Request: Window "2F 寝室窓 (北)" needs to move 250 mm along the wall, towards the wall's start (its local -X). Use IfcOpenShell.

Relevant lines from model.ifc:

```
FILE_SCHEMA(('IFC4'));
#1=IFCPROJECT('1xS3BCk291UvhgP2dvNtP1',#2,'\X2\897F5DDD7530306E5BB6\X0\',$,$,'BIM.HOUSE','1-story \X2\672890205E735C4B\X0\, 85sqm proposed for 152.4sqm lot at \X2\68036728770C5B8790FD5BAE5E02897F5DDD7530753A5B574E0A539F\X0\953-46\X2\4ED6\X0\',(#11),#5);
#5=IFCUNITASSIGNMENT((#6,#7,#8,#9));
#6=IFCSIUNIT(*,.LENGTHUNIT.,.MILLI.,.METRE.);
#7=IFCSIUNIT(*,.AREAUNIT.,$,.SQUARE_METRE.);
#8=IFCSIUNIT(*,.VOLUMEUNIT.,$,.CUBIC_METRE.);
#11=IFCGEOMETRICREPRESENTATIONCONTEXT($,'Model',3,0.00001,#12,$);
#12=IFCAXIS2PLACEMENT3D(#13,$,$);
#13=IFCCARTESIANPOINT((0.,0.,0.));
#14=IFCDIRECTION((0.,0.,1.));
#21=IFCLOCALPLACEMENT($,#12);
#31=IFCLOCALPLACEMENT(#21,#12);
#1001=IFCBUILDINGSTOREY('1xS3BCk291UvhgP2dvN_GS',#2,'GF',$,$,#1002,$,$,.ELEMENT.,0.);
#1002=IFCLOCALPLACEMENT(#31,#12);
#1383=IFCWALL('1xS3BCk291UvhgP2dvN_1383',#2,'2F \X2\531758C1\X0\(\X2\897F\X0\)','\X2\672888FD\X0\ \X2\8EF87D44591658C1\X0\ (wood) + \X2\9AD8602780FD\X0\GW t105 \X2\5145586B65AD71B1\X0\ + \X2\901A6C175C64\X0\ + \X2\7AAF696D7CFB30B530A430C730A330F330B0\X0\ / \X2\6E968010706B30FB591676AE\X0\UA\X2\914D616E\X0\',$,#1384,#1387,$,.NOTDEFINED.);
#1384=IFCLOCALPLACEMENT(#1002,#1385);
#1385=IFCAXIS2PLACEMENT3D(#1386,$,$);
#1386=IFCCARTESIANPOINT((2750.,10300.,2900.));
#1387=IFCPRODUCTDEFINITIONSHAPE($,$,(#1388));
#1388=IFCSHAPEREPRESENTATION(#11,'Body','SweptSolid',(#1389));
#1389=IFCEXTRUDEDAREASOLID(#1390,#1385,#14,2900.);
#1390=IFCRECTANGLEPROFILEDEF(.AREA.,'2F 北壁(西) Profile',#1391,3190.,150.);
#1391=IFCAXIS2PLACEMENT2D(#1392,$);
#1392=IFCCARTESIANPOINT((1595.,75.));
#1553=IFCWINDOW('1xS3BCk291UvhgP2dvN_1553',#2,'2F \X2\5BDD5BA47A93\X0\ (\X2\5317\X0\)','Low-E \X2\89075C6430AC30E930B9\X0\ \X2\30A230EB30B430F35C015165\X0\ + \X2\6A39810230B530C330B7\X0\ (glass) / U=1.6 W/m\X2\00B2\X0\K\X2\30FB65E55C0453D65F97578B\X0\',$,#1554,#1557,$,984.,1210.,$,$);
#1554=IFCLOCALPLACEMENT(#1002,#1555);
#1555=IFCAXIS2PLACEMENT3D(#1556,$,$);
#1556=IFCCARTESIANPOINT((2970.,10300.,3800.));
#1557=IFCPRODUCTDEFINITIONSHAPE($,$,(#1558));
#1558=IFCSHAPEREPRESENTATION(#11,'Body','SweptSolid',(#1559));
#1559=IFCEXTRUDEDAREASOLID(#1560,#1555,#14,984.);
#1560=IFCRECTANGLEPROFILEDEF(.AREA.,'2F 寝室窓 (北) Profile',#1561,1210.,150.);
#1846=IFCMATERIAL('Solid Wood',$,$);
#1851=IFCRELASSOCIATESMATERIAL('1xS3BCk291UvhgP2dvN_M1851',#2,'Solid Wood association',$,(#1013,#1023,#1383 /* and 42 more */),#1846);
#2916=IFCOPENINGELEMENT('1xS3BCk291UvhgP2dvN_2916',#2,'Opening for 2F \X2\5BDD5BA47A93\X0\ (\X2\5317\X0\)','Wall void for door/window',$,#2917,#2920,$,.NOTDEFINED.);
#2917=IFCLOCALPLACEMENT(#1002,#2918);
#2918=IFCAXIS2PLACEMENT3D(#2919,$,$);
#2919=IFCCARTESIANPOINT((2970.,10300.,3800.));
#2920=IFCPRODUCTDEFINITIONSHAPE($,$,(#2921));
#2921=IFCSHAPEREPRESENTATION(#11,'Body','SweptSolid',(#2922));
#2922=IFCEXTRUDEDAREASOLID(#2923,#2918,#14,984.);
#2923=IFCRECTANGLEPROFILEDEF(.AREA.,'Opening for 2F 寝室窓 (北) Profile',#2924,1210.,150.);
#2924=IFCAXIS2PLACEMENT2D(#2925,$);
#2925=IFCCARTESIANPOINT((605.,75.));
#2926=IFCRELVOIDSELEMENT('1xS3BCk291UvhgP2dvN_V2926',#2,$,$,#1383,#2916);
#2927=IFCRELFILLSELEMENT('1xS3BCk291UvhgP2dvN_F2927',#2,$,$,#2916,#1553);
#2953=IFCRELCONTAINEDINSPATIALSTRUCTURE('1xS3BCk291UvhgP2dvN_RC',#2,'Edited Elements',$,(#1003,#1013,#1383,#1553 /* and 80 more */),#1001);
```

```python
import ifcopenshell
import ifcopenshell.api.geometry
import ifcopenshell.util.placement
import ifcopenshell.util.unit

model = ifcopenshell.open("model.ifc")
unit_scale = ifcopenshell.util.unit.calculate_unit_scale(model)

window = model.by_id(1553)
opening = window.FillsVoids[0].RelatingOpeningElement
wall = opening.VoidsElements[0].RelatingBuildingElement

wall_matrix = ifcopenshell.util.placement.get_local_placement(wall.ObjectPlacement)
shift = wall_matrix[:3, 0] * -0.25 / unit_scale
before = ifcopenshell.util.placement.get_local_placement(window.ObjectPlacement)[:3, 3].copy()

# The window is not placed relative to its opening, so move both.
for product in (opening, window):
    matrix = ifcopenshell.util.placement.get_local_placement(product.ObjectPlacement)
    matrix[:3, 3] += shift
    ifcopenshell.api.geometry.edit_object_placement(model, product=product, matrix=matrix, is_si=False)

after = ifcopenshell.util.placement.get_local_placement(window.ObjectPlacement)[:3, 3]
print("window moved by", (after - before).round(3) + 0.0)

model.write("model_edited.ifc")
```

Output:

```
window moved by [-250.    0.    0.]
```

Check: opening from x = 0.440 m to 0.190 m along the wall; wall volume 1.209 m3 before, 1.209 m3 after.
